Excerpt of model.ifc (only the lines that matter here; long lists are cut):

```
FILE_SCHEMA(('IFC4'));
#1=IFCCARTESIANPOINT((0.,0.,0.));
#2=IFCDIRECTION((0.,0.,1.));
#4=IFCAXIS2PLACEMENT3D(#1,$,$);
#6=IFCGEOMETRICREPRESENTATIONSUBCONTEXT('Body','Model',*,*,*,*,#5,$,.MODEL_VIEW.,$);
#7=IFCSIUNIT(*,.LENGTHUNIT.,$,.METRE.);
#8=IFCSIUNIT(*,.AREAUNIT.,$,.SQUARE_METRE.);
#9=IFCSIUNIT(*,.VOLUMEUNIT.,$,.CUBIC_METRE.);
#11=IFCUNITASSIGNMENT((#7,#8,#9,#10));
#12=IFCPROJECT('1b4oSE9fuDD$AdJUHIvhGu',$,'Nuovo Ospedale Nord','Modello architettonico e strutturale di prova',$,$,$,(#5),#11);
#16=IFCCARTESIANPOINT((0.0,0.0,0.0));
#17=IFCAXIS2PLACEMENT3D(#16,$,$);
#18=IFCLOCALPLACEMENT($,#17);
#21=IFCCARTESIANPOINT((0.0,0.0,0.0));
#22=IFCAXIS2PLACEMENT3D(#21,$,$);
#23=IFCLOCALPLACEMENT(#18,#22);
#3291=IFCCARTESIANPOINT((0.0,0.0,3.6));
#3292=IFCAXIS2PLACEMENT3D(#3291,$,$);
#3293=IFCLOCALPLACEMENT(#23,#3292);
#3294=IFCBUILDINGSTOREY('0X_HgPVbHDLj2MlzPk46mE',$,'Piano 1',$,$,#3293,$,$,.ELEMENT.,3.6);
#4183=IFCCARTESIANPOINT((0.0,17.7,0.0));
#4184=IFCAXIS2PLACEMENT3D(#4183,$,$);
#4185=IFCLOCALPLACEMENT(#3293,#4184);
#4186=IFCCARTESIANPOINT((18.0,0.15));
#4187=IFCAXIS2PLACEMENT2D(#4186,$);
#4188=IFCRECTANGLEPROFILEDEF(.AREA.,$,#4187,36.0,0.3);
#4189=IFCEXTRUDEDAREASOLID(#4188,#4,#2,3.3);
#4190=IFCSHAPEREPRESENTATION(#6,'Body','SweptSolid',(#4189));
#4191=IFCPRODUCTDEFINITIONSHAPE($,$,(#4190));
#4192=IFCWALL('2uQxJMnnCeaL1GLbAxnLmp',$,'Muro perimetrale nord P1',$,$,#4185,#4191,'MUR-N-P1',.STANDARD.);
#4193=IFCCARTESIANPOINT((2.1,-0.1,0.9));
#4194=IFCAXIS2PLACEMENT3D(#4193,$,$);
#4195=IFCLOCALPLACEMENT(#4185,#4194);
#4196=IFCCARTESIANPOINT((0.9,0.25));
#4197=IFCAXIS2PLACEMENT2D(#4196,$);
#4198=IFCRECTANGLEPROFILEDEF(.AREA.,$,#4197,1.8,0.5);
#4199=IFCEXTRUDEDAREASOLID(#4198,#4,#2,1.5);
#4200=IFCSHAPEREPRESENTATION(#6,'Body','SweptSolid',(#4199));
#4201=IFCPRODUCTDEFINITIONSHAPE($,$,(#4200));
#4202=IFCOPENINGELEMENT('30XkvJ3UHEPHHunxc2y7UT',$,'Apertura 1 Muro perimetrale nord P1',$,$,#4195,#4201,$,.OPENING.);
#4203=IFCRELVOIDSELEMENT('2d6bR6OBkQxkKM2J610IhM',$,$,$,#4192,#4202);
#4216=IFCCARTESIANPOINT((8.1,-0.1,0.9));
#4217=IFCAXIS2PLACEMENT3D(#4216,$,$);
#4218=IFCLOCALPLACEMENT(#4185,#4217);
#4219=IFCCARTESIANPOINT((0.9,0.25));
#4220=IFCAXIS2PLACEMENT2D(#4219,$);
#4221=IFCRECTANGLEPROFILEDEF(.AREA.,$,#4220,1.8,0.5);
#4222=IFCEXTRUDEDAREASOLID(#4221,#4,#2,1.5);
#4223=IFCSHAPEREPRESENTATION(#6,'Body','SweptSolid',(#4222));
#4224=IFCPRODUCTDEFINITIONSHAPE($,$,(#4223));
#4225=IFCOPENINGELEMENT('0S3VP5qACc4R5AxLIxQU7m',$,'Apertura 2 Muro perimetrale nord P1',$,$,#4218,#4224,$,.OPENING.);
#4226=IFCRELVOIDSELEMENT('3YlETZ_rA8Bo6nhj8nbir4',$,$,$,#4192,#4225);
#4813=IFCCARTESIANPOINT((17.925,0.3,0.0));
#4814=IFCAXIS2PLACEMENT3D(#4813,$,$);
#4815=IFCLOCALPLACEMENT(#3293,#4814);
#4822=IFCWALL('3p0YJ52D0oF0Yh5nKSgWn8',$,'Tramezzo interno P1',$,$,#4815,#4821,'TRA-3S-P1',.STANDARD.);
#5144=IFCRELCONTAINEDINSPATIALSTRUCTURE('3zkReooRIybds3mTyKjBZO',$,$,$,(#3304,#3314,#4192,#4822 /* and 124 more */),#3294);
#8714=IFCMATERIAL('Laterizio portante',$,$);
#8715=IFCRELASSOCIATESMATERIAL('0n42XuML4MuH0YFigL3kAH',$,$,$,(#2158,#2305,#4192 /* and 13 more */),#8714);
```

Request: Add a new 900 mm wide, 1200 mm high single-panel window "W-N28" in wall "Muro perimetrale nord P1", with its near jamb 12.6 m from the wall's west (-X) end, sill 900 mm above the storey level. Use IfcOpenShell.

```python
import numpy as np
import ifcopenshell
import ifcopenshell.api.feature
import ifcopenshell.api.geometry
import ifcopenshell.api.root
import ifcopenshell.api.spatial
import ifcopenshell.geom
import ifcopenshell.util.element
import ifcopenshell.util.placement
import ifcopenshell.util.representation
import ifcopenshell.util.shape
import ifcopenshell.util.unit

model = ifcopenshell.open("model.ifc")
unit_scale = ifcopenshell.util.unit.calculate_unit_scale(model)
settings = ifcopenshell.geom.settings()


def volume(element):
    """Net volume in cubic metres, openings subtracted."""
    shape = ifcopenshell.geom.create_shape(settings, element)
    return ifcopenshell.util.shape.get_volume(shape.geometry)


wall = model.by_guid("2uQxJMnnCeaL1GLbAxnLmp")
storey = ifcopenshell.util.element.get_container(wall, ifc_class="IfcBuildingStorey")
context = ifcopenshell.util.representation.get_context(model, "Model", "Body", "MODEL_VIEW")
before = volume(wall)

width, height, from_end, sill = 0.9, 1.2, 12.6, 0.9  # metres

# The wall runs along its own X axis, and the end named is its -X end.
wall_shape = ifcopenshell.geom.create_shape(settings, wall)
x, y, z = ifcopenshell.util.shape.get_vertices(wall_shape.geometry).T
start = x.min() + from_end
face, thickness = float(y.min()), float(y.max() - y.min())
wall_matrix = ifcopenshell.util.placement.get_local_placement(wall.ObjectPlacement)
level = ifcopenshell.util.placement.get_local_placement(storey.ObjectPlacement)[2, 3]


def in_wall(x, y):
    """Placement at x, y metres in the wall's axes, at sill height."""
    matrix = wall_matrix.copy()
    matrix[:, 3] = wall_matrix @ np.array([x / unit_scale, y / unit_scale, 0.0, 1.0])
    matrix[2, 3] = level + sill / unit_scale
    return matrix


# Opening: a box that overshoots both wall faces by 50 mm.
opening = ifcopenshell.api.root.create_entity(model, ifc_class="IfcOpeningElement", predefined_type="OPENING")
box = ifcopenshell.api.geometry.add_wall_representation(
    model, context=context, length=width, height=height, thickness=thickness + 0.1
)
ifcopenshell.api.geometry.assign_representation(model, product=opening, representation=box)
ifcopenshell.api.geometry.edit_object_placement(model, product=opening, matrix=in_wall(start, face - 0.05), is_si=False)
ifcopenshell.api.feature.add_feature(model, feature=opening, element=wall)

window = ifcopenshell.api.root.create_entity(model, ifc_class="IfcWindow", name="W-N28", predefined_type="WINDOW")
window.OverallWidth, window.OverallHeight = width / unit_scale, height / unit_scale
window.PartitioningType = "SINGLE_PANEL"
body = ifcopenshell.api.geometry.add_window_representation(
    model,
    context=context,
    overall_width=window.OverallWidth,
    overall_height=window.OverallHeight,
    partition_type="SINGLE_PANEL",
)
ifcopenshell.api.geometry.assign_representation(model, product=window, representation=body)
ifcopenshell.api.spatial.assign_container(model, products=[window], relating_structure=storey)
ifcopenshell.api.feature.add_filling(model, opening=opening, element=window)

# Centre the window in the wall's thickness.
ifcopenshell.api.geometry.edit_object_placement(model, product=window, matrix=in_wall(start, face), is_si=False)
window_shape = ifcopenshell.geom.create_shape(settings, window)
depth = ifcopenshell.util.shape.get_vertices(window_shape.geometry)[:, 1]
offset = face + thickness / 2 - (depth.min() + depth.max()) / 2
ifcopenshell.api.geometry.edit_object_placement(model, product=window, matrix=in_wall(start, offset), is_si=False)

after = volume(wall)

print(f"wall volume {before:.3f} -> {after:.3f} m3")

model.write("model_updated.ifc")
```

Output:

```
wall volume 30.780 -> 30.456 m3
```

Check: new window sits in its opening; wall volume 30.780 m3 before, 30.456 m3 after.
